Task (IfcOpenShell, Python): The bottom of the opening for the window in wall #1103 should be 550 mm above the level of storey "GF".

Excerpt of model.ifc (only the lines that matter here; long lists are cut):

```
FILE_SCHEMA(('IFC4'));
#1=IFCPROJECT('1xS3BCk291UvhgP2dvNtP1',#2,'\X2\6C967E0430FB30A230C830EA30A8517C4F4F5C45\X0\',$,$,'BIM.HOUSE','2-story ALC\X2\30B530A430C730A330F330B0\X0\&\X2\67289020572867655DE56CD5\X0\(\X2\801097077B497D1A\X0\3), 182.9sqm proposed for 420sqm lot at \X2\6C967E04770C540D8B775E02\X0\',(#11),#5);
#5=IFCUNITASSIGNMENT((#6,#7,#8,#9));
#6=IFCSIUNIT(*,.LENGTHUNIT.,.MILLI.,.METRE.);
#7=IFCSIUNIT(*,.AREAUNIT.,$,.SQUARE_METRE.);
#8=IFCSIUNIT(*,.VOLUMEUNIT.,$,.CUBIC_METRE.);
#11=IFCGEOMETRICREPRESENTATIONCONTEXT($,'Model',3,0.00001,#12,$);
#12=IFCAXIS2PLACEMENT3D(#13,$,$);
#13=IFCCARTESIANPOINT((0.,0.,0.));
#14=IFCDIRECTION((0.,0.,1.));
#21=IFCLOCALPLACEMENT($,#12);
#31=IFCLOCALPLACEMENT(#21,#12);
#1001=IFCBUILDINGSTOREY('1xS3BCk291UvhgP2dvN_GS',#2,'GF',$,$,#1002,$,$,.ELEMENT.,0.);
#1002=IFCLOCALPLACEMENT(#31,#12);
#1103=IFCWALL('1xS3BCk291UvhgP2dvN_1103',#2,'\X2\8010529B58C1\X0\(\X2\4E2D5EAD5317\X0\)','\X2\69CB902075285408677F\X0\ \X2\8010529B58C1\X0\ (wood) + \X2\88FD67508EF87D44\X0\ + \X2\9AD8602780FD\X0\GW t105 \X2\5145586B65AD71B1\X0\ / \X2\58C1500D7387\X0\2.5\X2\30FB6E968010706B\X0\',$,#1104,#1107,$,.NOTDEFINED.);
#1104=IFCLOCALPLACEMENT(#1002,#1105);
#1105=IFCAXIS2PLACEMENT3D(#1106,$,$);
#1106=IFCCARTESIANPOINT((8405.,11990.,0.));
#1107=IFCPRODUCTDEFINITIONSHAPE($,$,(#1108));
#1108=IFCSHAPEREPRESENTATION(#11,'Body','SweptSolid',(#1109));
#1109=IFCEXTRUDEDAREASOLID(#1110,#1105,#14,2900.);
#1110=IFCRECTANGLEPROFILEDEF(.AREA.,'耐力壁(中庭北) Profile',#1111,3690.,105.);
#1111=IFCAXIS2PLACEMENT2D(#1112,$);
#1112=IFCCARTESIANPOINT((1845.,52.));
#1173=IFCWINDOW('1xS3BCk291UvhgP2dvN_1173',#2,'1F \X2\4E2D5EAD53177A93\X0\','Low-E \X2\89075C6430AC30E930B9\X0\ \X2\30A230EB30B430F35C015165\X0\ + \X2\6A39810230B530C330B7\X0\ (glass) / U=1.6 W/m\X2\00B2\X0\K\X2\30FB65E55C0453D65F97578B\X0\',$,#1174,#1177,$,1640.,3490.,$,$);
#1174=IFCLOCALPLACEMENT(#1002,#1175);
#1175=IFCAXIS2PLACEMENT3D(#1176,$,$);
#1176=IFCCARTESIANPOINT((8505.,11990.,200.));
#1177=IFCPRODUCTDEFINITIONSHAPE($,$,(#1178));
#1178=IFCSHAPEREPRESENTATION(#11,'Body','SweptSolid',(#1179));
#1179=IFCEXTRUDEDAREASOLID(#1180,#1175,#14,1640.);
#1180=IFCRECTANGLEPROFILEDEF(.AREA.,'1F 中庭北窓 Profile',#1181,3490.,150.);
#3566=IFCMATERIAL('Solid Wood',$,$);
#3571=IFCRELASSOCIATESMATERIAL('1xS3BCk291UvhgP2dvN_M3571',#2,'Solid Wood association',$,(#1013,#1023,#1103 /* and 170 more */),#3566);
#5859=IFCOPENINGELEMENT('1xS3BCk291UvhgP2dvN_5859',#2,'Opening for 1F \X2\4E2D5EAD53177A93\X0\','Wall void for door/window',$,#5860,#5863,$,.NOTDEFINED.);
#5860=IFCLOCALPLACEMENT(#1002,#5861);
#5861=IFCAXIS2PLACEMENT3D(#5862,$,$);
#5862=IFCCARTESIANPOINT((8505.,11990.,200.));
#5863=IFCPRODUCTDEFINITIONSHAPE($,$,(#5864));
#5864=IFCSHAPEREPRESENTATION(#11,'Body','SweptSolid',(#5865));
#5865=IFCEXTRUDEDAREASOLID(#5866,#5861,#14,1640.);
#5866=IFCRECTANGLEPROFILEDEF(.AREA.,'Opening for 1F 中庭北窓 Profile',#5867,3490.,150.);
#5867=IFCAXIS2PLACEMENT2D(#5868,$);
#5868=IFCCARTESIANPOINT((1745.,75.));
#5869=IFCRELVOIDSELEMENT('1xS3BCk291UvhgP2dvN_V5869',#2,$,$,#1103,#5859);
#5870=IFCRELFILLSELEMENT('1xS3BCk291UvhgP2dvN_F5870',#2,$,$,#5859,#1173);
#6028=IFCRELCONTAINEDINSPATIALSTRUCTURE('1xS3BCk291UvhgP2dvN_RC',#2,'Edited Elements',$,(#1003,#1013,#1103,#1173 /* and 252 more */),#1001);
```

```python
import numpy as np
import ifcopenshell
import ifcopenshell.api.geometry
import ifcopenshell.geom
import ifcopenshell.util.element
import ifcopenshell.util.placement
import ifcopenshell.util.shape
import ifcopenshell.util.unit

model = ifcopenshell.open("model.ifc")
unit_scale = ifcopenshell.util.unit.calculate_unit_scale(model)

window = model.by_guid("1xS3BCk291UvhgP2dvN_1173")
opening = window.FillsVoids[0].RelatingOpeningElement
storey = ifcopenshell.util.element.get_container(window, ifc_class="IfcBuildingStorey")
level = ifcopenshell.util.placement.get_local_placement(storey.ObjectPlacement)[2, 3]

# The opening's origin need not be at the sill, so measure its lowest point.
shape = ifcopenshell.geom.create_shape(ifcopenshell.geom.settings(), opening)
bottom = ifcopenshell.util.shape.get_shape_bottom_elevation(shape, shape.geometry) / unit_scale
dz = level + 550.0 - bottom

shift = np.array([0.0, 0.0, dz])
# The window is not placed relative to its opening, so move both.
for product in (opening, window):
    matrix = ifcopenshell.util.placement.get_local_placement(product.ObjectPlacement)
    matrix[:3, 3] += shift
    ifcopenshell.api.geometry.edit_object_placement(model, product=product, matrix=matrix, is_si=False)

print(f"moved by {dz * unit_scale:+.3f} m")

model.write("model_v2.ifc")
```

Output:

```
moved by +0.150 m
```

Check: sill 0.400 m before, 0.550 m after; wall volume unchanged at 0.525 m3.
